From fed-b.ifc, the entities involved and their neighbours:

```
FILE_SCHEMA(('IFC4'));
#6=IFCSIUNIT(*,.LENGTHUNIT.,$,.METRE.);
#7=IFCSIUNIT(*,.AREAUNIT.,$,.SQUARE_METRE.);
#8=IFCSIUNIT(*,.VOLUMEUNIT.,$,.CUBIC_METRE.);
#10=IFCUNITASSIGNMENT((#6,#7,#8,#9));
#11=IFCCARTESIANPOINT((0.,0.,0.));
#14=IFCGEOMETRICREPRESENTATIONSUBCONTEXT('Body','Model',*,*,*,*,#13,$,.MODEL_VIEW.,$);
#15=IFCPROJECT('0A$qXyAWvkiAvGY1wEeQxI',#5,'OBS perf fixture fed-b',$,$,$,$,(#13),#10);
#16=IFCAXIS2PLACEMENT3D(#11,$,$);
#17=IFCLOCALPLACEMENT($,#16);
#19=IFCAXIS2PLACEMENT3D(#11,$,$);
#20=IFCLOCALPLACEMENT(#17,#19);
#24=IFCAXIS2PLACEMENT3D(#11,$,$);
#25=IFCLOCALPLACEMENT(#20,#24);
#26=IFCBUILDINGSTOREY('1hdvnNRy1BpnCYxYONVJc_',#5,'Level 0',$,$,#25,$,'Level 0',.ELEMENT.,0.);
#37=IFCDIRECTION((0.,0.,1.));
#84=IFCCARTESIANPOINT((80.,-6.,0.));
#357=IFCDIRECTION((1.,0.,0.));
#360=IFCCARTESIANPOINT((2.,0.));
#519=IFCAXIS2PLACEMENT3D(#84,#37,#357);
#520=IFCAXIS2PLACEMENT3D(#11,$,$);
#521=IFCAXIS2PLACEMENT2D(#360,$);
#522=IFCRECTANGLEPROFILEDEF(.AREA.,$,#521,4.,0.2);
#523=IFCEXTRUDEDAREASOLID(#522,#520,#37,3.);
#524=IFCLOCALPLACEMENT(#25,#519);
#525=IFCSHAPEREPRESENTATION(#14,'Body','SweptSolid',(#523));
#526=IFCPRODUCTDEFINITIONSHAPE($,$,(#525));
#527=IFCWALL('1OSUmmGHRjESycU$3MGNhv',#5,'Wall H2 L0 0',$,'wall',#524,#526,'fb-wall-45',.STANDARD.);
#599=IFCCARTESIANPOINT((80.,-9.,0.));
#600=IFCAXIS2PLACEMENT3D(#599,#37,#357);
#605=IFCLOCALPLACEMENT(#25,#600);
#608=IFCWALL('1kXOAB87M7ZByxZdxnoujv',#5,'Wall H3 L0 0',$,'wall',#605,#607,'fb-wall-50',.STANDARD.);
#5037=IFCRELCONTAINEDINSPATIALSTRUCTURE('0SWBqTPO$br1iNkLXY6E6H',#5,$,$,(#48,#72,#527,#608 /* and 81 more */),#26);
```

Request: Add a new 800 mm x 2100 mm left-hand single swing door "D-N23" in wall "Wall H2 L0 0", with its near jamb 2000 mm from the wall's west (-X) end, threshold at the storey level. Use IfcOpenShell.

```python
import numpy as np
import ifcopenshell
import ifcopenshell.api.feature
import ifcopenshell.api.geometry
import ifcopenshell.api.root
import ifcopenshell.api.spatial
import ifcopenshell.geom
import ifcopenshell.util.element
import ifcopenshell.util.placement
import ifcopenshell.util.representation
import ifcopenshell.util.shape
import ifcopenshell.util.unit

model = ifcopenshell.open("fed-b.ifc")
unit_scale = ifcopenshell.util.unit.calculate_unit_scale(model)
settings = ifcopenshell.geom.settings()


def volume(element):
    """Net volume in cubic metres, openings subtracted."""
    shape = ifcopenshell.geom.create_shape(settings, element)
    return ifcopenshell.util.shape.get_volume(shape.geometry)


wall = model.by_guid("1OSUmmGHRjESycU$3MGNhv")
storey = ifcopenshell.util.element.get_container(wall, ifc_class="IfcBuildingStorey")
context = ifcopenshell.util.representation.get_context(model, "Model", "Body", "MODEL_VIEW")
before = volume(wall)

width, height, from_end, sill = 0.8, 2.1, 2, 0.0  # metres

# The wall runs along its own X axis, and the end named is its -X end.
wall_shape = ifcopenshell.geom.create_shape(settings, wall)
x, y, z = ifcopenshell.util.shape.get_vertices(wall_shape.geometry).T
start = x.min() + from_end
face, thickness = float(y.min()), float(y.max() - y.min())
wall_matrix = ifcopenshell.util.placement.get_local_placement(wall.ObjectPlacement)
level = ifcopenshell.util.placement.get_local_placement(storey.ObjectPlacement)[2, 3]


def in_wall(x, y):
    """Placement at x, y metres in the wall's axes, at sill height."""
    matrix = wall_matrix.copy()
    matrix[:, 3] = wall_matrix @ np.array([x / unit_scale, y / unit_scale, 0.0, 1.0])
    matrix[2, 3] = level + sill / unit_scale
    return matrix


# Opening: a box that overshoots both wall faces by 50 mm.
opening = ifcopenshell.api.root.create_entity(model, ifc_class="IfcOpeningElement", predefined_type="OPENING")
box = ifcopenshell.api.geometry.add_wall_representation(
    model, context=context, length=width, height=height, thickness=thickness + 0.1
)
ifcopenshell.api.geometry.assign_representation(model, product=opening, representation=box)
ifcopenshell.api.geometry.edit_object_placement(model, product=opening, matrix=in_wall(start, face - 0.05), is_si=False)
ifcopenshell.api.feature.add_feature(model, feature=opening, element=wall)

door = ifcopenshell.api.root.create_entity(model, ifc_class="IfcDoor", name="D-N23", predefined_type="DOOR")
door.OverallWidth, door.OverallHeight = width / unit_scale, height / unit_scale
door.OperationType = "SINGLE_SWING_LEFT"
body = ifcopenshell.api.geometry.add_door_representation(
    model,
    context=context,
    overall_width=door.OverallWidth,
    overall_height=door.OverallHeight,
    operation_type="SINGLE_SWING_LEFT",
    lining_properties={"LiningDepth": thickness / unit_scale, "ThresholdDepth": thickness / unit_scale},
)
ifcopenshell.api.geometry.assign_representation(model, product=door, representation=body)
ifcopenshell.api.spatial.assign_container(model, products=[door], relating_structure=storey)
ifcopenshell.api.feature.add_filling(model, opening=opening, element=door)

# The lining spans the wall, so the door starts at the wall face.
ifcopenshell.api.geometry.edit_object_placement(model, product=door, matrix=in_wall(start, face), is_si=False)

after = volume(wall)

print(f"wall volume {before:.3f} -> {after:.3f} m3")

model.write("fed-b_v2.ifc")
```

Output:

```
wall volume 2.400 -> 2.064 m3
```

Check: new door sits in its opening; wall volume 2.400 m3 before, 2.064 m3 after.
